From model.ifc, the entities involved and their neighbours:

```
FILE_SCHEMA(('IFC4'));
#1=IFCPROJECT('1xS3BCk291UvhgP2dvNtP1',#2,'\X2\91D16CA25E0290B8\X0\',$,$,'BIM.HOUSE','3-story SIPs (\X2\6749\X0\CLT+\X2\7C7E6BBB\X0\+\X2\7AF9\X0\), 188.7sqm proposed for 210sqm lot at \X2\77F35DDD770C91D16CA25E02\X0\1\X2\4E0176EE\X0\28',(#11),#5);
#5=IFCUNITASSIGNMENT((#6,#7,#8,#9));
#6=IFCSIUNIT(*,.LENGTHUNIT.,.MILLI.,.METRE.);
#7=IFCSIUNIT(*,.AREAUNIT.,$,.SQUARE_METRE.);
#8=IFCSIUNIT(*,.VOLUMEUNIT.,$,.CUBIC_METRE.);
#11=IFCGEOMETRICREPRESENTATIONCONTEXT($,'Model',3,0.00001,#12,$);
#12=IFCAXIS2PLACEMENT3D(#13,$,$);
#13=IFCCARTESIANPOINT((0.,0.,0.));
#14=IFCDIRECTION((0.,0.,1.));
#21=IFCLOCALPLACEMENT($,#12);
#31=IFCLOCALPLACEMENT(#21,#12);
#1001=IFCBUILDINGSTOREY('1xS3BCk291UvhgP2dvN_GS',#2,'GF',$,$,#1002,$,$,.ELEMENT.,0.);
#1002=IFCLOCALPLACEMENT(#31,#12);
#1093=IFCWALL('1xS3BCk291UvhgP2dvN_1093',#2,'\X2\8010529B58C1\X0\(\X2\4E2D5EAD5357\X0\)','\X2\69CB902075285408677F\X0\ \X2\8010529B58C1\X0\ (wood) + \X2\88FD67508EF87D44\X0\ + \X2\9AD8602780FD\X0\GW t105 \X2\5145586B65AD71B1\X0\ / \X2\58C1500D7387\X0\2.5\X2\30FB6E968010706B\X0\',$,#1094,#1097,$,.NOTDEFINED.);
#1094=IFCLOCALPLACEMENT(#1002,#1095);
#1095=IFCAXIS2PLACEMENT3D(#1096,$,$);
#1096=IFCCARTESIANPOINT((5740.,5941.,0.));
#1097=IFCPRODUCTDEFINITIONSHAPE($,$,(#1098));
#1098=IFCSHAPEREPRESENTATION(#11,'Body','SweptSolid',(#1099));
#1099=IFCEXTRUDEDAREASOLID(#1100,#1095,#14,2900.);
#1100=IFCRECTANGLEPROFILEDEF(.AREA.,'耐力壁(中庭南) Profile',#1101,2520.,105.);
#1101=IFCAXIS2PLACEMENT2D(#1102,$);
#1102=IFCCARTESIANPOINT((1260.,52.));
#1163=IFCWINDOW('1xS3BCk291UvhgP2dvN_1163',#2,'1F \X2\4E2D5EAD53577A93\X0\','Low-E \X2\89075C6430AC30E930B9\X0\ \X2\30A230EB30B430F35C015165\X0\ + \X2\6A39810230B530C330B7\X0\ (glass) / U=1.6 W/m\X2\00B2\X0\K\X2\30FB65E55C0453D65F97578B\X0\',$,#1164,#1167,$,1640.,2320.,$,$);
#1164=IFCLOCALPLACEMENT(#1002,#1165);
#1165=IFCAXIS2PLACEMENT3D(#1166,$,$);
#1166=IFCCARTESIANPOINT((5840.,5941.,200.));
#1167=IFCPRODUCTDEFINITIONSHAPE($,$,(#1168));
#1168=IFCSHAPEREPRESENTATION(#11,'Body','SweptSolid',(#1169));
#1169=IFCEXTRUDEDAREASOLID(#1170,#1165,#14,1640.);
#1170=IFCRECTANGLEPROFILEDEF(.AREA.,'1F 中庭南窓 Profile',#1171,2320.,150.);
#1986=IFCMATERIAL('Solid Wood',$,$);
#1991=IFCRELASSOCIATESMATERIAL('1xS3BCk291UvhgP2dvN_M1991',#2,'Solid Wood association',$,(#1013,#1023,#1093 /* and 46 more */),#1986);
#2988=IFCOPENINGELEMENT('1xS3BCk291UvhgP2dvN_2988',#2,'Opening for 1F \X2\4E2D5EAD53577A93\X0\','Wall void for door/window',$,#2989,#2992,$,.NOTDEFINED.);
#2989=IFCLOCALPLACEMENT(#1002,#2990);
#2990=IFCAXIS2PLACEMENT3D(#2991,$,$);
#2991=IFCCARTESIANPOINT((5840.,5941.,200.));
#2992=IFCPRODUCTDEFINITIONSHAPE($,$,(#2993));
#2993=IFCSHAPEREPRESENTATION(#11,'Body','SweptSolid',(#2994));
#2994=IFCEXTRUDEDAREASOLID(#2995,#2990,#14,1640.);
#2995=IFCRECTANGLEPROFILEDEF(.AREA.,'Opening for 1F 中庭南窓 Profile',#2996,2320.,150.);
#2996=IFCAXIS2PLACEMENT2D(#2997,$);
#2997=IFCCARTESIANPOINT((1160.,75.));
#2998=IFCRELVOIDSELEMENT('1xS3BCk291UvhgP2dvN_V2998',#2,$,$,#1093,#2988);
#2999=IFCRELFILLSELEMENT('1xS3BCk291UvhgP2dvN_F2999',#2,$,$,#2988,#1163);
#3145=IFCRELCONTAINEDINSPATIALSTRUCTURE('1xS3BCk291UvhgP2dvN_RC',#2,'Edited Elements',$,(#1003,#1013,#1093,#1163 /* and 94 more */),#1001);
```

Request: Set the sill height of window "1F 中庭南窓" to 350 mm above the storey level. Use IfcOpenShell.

```python
import numpy as np
import ifcopenshell
import ifcopenshell.api.geometry
import ifcopenshell.geom
import ifcopenshell.util.element
import ifcopenshell.util.placement
import ifcopenshell.util.shape
import ifcopenshell.util.unit

model = ifcopenshell.open("model.ifc")
unit_scale = ifcopenshell.util.unit.calculate_unit_scale(model)

window = model.by_guid("1xS3BCk291UvhgP2dvN_1163")
opening = window.FillsVoids[0].RelatingOpeningElement
storey = ifcopenshell.util.element.get_container(window, ifc_class="IfcBuildingStorey")
level = ifcopenshell.util.placement.get_local_placement(storey.ObjectPlacement)[2, 3]

# The opening's origin need not be at the sill, so measure its lowest point.
shape = ifcopenshell.geom.create_shape(ifcopenshell.geom.settings(), opening)
bottom = ifcopenshell.util.shape.get_shape_bottom_elevation(shape, shape.geometry) / unit_scale
dz = level + 350.0 - bottom

shift = np.array([0.0, 0.0, dz])
# The window is not placed relative to its opening, so move both.
for product in (opening, window):
    matrix = ifcopenshell.util.placement.get_local_placement(product.ObjectPlacement)
    matrix[:3, 3] += shift
    ifcopenshell.api.geometry.edit_object_placement(model, product=product, matrix=matrix, is_si=False)

print(f"moved by {dz * unit_scale:+.3f} m")

model.write("model_updated.ifc")
```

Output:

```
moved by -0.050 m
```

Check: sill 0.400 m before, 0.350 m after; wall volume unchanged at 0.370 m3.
